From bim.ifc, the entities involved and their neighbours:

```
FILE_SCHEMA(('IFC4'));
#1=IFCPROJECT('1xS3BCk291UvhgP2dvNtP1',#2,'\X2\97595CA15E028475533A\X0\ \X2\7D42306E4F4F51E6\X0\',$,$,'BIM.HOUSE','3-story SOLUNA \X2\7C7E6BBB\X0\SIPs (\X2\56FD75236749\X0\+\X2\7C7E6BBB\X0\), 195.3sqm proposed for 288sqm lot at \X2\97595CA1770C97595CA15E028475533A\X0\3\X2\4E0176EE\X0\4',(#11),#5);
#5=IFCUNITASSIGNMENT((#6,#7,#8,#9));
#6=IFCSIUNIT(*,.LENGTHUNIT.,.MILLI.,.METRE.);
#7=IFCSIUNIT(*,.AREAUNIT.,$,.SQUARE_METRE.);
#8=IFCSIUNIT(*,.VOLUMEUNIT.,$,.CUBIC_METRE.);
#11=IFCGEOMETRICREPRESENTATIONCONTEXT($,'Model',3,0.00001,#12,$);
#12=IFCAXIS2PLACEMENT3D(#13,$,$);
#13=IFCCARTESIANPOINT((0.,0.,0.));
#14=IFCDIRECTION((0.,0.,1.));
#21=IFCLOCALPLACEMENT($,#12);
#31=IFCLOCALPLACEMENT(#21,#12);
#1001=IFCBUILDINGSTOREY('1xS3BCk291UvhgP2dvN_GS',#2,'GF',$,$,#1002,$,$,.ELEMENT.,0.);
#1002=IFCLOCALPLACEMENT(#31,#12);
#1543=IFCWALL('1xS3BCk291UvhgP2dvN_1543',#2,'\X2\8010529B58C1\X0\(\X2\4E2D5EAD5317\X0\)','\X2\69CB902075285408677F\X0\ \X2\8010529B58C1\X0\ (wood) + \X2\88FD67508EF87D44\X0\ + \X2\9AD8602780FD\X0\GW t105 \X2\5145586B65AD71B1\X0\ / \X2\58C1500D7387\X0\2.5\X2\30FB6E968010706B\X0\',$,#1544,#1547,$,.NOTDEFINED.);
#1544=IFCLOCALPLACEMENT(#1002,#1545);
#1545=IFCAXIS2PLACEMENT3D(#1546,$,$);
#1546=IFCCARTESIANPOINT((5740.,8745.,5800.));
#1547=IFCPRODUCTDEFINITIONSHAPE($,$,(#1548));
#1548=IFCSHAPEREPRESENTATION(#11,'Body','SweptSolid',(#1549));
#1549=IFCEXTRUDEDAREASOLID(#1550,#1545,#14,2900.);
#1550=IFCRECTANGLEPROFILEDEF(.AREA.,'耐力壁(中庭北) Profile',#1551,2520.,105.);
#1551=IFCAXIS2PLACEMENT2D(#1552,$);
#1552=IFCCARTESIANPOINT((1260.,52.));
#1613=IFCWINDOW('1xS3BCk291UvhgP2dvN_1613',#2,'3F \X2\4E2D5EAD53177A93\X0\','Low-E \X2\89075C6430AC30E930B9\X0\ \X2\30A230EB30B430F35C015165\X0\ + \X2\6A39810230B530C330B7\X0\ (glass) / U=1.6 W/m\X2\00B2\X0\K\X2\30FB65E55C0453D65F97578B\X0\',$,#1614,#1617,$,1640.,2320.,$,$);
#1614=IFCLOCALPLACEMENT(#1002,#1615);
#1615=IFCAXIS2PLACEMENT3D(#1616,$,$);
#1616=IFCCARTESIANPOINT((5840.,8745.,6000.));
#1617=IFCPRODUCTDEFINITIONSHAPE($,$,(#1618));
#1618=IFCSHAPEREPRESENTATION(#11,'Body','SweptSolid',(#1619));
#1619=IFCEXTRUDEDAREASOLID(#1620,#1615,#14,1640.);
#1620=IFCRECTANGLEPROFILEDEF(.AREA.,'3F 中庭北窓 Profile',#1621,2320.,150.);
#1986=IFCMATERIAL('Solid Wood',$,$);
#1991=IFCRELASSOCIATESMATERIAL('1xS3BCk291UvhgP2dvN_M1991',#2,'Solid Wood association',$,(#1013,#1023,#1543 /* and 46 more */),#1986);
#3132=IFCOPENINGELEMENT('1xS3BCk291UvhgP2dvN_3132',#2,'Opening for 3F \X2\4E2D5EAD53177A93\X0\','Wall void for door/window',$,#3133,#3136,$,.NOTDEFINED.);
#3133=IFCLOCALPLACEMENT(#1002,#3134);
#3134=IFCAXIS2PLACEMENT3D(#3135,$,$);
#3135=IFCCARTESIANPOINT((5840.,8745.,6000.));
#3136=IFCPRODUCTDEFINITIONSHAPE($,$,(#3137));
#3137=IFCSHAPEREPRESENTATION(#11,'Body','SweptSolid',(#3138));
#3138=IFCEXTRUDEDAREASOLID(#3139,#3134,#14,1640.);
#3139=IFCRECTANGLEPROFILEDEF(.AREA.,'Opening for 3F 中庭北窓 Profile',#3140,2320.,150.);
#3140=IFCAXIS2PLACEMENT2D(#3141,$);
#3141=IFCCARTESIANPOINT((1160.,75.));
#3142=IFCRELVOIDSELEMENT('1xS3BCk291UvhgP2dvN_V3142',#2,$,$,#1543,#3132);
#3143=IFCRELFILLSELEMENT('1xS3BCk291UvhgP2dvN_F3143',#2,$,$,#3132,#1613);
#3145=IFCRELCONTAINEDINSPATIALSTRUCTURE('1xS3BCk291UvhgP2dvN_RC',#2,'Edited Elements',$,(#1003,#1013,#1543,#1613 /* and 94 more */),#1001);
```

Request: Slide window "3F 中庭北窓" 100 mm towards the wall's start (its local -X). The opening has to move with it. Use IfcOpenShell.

```python
import ifcopenshell
import ifcopenshell.api.geometry
import ifcopenshell.util.placement

model = ifcopenshell.open("bim.ifc")

window = model.by_id(1613)
opening = window.FillsVoids[0].RelatingOpeningElement
wall = opening.VoidsElements[0].RelatingBuildingElement

wall_matrix = ifcopenshell.util.placement.get_local_placement(wall.ObjectPlacement)
shift = wall_matrix[:3, 0] * -100.0
before = ifcopenshell.util.placement.get_local_placement(window.ObjectPlacement)[:3, 3].copy()

# The window is not placed relative to its opening, so move both.
for product in (opening, window):
    matrix = ifcopenshell.util.placement.get_local_placement(product.ObjectPlacement)
    matrix[:3, 3] += shift
    ifcopenshell.api.geometry.edit_object_placement(model, product=product, matrix=matrix, is_si=False)

after = ifcopenshell.util.placement.get_local_placement(window.ObjectPlacement)[:3, 3]
print("window moved by", (after - before).round(3) + 0.0)

model.write("bim-out.ifc")
```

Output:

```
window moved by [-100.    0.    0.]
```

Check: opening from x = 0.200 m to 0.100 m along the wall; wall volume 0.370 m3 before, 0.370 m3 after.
